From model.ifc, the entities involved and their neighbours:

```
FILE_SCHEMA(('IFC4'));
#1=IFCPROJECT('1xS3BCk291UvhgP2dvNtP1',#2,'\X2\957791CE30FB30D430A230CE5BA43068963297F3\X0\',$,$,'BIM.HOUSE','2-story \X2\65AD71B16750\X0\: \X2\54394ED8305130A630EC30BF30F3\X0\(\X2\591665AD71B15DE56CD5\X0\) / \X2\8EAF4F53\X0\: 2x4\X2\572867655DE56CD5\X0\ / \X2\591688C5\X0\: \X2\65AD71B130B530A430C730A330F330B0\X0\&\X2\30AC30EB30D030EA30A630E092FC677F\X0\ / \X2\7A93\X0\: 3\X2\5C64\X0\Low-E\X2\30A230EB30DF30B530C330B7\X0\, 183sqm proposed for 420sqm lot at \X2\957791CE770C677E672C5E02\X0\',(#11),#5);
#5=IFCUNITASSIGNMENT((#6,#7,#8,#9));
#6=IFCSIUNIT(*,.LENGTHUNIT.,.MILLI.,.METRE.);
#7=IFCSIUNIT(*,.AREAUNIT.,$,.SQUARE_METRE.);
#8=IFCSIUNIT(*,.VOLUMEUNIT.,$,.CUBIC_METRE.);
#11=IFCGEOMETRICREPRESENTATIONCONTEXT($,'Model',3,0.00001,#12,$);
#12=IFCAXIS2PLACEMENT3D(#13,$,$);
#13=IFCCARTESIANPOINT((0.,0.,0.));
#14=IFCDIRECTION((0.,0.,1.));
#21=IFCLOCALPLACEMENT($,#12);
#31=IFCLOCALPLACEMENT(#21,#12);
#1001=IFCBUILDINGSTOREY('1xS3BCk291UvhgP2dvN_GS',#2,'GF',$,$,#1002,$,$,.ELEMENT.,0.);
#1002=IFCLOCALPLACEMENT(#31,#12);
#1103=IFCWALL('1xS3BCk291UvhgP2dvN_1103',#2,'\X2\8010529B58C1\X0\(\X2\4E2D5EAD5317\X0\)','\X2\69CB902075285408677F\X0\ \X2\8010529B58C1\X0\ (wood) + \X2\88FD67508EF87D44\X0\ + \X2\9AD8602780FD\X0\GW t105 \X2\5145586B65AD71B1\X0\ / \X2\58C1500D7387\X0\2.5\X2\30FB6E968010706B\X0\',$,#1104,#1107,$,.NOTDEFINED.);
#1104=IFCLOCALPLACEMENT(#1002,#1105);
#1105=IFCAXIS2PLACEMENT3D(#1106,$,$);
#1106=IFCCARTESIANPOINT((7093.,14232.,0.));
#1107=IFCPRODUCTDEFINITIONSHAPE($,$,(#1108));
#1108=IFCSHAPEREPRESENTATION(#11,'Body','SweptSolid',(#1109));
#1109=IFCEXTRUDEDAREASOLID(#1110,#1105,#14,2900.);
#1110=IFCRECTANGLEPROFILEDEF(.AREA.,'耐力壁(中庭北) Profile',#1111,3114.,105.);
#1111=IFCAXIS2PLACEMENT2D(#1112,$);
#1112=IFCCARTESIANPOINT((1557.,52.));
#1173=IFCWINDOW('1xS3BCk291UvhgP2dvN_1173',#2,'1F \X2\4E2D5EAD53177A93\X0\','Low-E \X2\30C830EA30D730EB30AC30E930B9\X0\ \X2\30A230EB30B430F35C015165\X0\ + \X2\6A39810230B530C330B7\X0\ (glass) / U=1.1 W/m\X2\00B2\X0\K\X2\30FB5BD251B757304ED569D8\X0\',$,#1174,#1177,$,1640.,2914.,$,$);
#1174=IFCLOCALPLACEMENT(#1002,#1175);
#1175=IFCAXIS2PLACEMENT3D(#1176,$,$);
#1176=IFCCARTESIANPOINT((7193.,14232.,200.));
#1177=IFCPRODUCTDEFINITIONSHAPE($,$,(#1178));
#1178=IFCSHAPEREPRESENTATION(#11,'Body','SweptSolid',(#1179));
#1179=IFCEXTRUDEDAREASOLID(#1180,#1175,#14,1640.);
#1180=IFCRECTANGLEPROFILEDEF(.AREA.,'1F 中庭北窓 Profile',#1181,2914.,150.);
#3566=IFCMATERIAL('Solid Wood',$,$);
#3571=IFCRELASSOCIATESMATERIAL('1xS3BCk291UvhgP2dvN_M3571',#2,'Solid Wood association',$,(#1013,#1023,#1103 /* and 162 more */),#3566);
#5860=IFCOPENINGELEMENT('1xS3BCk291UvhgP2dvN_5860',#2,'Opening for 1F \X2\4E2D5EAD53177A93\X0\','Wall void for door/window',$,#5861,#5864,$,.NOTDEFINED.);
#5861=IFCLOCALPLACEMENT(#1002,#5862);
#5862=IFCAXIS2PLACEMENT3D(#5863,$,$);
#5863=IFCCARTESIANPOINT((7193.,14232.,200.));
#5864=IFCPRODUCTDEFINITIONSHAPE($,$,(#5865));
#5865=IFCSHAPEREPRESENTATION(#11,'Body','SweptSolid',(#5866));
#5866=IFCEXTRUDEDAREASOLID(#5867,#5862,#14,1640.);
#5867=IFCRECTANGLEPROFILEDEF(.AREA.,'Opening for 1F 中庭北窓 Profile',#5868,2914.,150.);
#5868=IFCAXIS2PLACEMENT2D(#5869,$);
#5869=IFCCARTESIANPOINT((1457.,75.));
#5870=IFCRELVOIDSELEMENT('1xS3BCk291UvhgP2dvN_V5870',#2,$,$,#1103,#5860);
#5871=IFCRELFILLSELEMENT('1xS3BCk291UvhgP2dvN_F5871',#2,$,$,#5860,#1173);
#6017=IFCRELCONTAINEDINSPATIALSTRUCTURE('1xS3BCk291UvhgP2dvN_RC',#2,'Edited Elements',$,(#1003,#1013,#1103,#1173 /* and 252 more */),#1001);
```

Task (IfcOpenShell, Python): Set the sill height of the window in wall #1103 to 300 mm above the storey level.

```python
import numpy as np
import ifcopenshell
import ifcopenshell.api.geometry
import ifcopenshell.geom
import ifcopenshell.util.element
import ifcopenshell.util.placement
import ifcopenshell.util.shape
import ifcopenshell.util.unit

model = ifcopenshell.open("model.ifc")
unit_scale = ifcopenshell.util.unit.calculate_unit_scale(model)

window = model.by_guid("1xS3BCk291UvhgP2dvN_1173")
opening = window.FillsVoids[0].RelatingOpeningElement
storey = ifcopenshell.util.element.get_container(window, ifc_class="IfcBuildingStorey")
level = ifcopenshell.util.placement.get_local_placement(storey.ObjectPlacement)[2, 3]

# The opening's origin need not be at the sill, so measure its lowest point.
shape = ifcopenshell.geom.create_shape(ifcopenshell.geom.settings(), opening)
bottom = ifcopenshell.util.shape.get_shape_bottom_elevation(shape, shape.geometry) / unit_scale
dz = level + 0.3 / unit_scale - bottom

shift = np.array([0.0, 0.0, dz])
# The window is not placed relative to its opening, so move both.
for product in (opening, window):
    matrix = ifcopenshell.util.placement.get_local_placement(product.ObjectPlacement)
    matrix[:3, 3] += shift
    ifcopenshell.api.geometry.edit_object_placement(model, product=product, matrix=matrix, is_si=False)

print(f"moved by {dz * unit_scale:+.3f} m")

model.write("model-out.ifc")
```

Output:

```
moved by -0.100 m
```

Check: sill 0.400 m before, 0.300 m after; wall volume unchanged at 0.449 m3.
